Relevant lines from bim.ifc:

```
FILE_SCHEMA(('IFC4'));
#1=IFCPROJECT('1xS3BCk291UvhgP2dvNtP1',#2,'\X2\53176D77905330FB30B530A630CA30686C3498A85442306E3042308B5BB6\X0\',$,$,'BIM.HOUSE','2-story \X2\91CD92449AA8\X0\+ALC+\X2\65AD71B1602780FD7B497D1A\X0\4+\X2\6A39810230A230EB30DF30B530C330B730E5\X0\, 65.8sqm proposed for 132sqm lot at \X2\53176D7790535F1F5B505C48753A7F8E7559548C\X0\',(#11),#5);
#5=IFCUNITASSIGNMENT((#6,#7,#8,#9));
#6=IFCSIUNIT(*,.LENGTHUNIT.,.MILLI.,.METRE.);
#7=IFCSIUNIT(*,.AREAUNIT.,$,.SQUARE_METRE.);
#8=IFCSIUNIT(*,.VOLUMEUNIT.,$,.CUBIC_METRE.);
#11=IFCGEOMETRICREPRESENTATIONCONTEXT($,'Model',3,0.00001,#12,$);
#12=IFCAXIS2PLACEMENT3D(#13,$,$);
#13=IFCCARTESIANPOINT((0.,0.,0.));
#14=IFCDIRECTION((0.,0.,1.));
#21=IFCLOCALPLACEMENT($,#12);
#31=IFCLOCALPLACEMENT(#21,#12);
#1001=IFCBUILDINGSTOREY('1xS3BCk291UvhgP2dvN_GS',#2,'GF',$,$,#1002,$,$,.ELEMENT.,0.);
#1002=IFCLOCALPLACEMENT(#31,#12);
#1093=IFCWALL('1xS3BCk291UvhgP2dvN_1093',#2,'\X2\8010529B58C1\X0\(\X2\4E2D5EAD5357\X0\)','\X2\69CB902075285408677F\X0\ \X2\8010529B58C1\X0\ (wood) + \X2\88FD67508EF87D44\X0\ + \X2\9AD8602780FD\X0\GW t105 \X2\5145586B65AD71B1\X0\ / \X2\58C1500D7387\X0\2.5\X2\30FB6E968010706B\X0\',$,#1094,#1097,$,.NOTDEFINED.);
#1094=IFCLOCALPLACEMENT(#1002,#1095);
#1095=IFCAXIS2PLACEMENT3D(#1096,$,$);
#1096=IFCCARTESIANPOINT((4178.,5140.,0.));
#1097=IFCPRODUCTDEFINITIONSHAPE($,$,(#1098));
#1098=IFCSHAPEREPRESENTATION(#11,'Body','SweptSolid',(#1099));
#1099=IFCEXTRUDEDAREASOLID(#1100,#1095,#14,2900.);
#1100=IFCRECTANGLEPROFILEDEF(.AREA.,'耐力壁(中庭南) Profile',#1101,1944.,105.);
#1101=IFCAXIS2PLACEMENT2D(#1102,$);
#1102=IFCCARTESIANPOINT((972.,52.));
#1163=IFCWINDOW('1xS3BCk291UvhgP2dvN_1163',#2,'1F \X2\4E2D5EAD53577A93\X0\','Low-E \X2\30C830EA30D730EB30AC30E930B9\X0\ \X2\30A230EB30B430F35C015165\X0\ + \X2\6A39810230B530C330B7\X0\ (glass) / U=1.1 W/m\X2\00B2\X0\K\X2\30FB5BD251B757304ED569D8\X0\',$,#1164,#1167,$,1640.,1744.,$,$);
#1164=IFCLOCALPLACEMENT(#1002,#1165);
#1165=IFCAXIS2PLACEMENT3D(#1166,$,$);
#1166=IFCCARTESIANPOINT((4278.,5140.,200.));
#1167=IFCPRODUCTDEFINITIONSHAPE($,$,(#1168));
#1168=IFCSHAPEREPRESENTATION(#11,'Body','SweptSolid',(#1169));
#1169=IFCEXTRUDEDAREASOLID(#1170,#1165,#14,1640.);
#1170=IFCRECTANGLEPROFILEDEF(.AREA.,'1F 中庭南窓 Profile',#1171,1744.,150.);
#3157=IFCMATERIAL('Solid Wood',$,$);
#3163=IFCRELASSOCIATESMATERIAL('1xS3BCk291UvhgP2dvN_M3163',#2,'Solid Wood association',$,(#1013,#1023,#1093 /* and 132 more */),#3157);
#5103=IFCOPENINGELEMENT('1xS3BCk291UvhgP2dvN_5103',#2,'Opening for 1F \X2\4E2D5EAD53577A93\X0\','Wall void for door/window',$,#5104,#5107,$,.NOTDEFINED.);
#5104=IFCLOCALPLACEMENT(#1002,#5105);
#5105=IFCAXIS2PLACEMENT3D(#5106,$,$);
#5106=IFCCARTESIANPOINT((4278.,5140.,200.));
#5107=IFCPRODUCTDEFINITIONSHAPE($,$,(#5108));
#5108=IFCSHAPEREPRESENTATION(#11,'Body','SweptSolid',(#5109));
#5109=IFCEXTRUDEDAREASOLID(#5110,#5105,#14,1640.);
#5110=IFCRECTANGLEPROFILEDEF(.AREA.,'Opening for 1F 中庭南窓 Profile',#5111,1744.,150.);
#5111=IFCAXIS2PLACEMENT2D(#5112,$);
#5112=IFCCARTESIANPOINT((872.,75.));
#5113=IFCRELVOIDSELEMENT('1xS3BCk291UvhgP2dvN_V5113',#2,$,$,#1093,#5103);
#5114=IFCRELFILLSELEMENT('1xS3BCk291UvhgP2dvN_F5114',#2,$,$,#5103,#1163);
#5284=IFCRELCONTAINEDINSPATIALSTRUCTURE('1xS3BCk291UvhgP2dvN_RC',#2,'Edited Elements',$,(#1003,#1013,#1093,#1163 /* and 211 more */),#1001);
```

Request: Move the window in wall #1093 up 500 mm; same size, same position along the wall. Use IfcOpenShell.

```python
import numpy as np
import ifcopenshell
import ifcopenshell.api.geometry
import ifcopenshell.util.placement
import ifcopenshell.util.unit

model = ifcopenshell.open("bim.ifc")
unit_scale = ifcopenshell.util.unit.calculate_unit_scale(model)

window = model.by_guid("1xS3BCk291UvhgP2dvN_1163")
opening = window.FillsVoids[0].RelatingOpeningElement
dz = 500.0

shift = np.array([0.0, 0.0, dz])
# The window is not placed relative to its opening, so move both.
for product in (opening, window):
    matrix = ifcopenshell.util.placement.get_local_placement(product.ObjectPlacement)
    matrix[:3, 3] += shift
    ifcopenshell.api.geometry.edit_object_placement(model, product=product, matrix=matrix, is_si=False)

print(f"moved by {dz * unit_scale:+.3f} m")

model.write("bim-out.ifc")
```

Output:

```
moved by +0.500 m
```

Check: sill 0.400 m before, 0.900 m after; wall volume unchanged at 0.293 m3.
